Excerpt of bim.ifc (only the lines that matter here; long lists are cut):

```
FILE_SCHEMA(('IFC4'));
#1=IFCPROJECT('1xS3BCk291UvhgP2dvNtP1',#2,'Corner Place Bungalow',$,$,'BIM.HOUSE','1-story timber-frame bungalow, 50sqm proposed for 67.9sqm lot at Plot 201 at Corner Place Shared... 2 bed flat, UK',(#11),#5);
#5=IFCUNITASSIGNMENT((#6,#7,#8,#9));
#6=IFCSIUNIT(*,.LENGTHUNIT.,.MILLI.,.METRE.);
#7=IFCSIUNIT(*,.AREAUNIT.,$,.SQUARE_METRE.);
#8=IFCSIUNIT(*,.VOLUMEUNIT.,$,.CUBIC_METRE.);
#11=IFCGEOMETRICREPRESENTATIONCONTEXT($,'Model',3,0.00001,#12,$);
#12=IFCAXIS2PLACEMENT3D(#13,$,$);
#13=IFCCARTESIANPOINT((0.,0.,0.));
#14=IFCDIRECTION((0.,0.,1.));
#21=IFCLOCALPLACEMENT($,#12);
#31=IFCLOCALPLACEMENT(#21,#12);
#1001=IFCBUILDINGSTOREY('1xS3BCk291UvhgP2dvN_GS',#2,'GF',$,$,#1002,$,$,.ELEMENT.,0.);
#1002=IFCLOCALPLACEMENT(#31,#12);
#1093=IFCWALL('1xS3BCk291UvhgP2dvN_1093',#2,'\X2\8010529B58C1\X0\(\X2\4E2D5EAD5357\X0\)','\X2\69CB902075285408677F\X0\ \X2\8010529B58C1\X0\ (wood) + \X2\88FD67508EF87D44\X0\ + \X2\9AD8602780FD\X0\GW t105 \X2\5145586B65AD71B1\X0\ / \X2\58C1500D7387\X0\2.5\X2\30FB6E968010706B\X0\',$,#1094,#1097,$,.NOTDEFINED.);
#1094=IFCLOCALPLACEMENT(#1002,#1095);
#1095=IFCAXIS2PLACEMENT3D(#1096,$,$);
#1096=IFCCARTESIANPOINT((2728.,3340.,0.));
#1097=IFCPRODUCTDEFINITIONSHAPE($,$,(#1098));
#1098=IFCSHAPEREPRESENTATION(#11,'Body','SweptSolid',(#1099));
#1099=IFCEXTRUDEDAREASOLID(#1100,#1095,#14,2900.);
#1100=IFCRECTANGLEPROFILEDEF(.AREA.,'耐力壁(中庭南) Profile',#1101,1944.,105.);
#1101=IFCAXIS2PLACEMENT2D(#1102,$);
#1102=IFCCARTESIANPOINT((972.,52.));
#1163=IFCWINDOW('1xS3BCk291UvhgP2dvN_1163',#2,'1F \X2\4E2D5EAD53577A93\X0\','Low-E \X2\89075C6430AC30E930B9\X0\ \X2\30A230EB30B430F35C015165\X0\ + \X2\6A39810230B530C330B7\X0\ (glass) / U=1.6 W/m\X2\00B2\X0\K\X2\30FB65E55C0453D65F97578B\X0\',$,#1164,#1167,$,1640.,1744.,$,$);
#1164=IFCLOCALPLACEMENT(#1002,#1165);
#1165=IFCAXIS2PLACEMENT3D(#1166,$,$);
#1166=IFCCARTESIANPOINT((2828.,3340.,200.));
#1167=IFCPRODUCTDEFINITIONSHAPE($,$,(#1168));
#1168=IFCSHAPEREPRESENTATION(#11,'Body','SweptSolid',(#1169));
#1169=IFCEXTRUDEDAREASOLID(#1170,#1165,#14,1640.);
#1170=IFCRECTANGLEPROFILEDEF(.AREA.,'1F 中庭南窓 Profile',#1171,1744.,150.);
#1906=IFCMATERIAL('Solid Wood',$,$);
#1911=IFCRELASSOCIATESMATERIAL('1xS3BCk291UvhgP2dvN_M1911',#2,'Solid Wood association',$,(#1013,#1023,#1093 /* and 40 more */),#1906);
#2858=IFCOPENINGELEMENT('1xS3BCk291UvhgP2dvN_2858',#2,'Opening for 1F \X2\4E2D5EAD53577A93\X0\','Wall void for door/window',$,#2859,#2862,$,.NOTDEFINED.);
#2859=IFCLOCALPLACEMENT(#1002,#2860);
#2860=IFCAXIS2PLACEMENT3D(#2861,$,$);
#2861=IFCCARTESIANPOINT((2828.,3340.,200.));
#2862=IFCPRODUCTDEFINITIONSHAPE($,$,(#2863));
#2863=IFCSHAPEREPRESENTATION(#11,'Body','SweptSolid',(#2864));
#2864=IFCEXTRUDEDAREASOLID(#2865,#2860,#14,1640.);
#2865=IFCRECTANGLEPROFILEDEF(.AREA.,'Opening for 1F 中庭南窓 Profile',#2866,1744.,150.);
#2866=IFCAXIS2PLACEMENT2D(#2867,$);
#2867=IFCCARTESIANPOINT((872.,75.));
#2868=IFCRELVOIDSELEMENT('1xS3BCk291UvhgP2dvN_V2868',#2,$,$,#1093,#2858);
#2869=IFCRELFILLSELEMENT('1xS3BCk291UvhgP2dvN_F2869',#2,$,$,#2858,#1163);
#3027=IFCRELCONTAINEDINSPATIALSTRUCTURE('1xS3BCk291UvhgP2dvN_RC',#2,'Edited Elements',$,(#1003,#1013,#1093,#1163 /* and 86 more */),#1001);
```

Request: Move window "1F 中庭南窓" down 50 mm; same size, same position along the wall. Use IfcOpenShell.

```python
import numpy as np
import ifcopenshell
import ifcopenshell.api.geometry
import ifcopenshell.util.placement
import ifcopenshell.util.unit

model = ifcopenshell.open("bim.ifc")
unit_scale = ifcopenshell.util.unit.calculate_unit_scale(model)

window = model.by_id(1163)
opening = window.FillsVoids[0].RelatingOpeningElement
dz = -0.05 / unit_scale

shift = np.array([0.0, 0.0, dz])
# The window is not placed relative to its opening, so move both.
for product in (opening, window):
    matrix = ifcopenshell.util.placement.get_local_placement(product.ObjectPlacement)
    matrix[:3, 3] += shift
    ifcopenshell.api.geometry.edit_object_placement(model, product=product, matrix=matrix, is_si=False)

print(f"moved by {dz * unit_scale:+.3f} m")

model.write("bim-out.ifc")
```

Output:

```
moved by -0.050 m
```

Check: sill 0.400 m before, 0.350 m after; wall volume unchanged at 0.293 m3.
